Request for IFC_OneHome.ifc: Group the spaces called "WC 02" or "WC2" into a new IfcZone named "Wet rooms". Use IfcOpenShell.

First a look at what the model holds.

```python
import ifcopenshell

model = ifcopenshell.open("IFC_OneHome.ifc")
print(model.schema)
seen = {}
for space in model.by_type("IfcSpace"):
    seen[space.LongName] = seen.get(space.LongName, 0) + 1
for name, count in sorted(seen.items(), key=str):
    print(count, "x", name)
print("zones:", [z.Name for z in model.by_type("IfcZone")][:20])
```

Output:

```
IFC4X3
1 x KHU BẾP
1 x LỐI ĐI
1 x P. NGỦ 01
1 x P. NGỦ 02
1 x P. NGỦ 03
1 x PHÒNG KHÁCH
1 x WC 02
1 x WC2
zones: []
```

```python
import ifcopenshell
import ifcopenshell.api.group
import ifcopenshell.api.root

model = ifcopenshell.open("IFC_OneHome.ifc")

names = {"WC 02", "WC2"}
spaces = [s for s in model.by_type("IfcSpace") if s.LongName in names]

zone = ifcopenshell.api.root.create_entity(model, ifc_class="IfcZone", name="Wet rooms")
ifcopenshell.api.group.assign_group(model, products=spaces, group=zone)
print(len(spaces), "spaces in", zone.Name)

model.write("IFC_OneHome_edited.ifc")
```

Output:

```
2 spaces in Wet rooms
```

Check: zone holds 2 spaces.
